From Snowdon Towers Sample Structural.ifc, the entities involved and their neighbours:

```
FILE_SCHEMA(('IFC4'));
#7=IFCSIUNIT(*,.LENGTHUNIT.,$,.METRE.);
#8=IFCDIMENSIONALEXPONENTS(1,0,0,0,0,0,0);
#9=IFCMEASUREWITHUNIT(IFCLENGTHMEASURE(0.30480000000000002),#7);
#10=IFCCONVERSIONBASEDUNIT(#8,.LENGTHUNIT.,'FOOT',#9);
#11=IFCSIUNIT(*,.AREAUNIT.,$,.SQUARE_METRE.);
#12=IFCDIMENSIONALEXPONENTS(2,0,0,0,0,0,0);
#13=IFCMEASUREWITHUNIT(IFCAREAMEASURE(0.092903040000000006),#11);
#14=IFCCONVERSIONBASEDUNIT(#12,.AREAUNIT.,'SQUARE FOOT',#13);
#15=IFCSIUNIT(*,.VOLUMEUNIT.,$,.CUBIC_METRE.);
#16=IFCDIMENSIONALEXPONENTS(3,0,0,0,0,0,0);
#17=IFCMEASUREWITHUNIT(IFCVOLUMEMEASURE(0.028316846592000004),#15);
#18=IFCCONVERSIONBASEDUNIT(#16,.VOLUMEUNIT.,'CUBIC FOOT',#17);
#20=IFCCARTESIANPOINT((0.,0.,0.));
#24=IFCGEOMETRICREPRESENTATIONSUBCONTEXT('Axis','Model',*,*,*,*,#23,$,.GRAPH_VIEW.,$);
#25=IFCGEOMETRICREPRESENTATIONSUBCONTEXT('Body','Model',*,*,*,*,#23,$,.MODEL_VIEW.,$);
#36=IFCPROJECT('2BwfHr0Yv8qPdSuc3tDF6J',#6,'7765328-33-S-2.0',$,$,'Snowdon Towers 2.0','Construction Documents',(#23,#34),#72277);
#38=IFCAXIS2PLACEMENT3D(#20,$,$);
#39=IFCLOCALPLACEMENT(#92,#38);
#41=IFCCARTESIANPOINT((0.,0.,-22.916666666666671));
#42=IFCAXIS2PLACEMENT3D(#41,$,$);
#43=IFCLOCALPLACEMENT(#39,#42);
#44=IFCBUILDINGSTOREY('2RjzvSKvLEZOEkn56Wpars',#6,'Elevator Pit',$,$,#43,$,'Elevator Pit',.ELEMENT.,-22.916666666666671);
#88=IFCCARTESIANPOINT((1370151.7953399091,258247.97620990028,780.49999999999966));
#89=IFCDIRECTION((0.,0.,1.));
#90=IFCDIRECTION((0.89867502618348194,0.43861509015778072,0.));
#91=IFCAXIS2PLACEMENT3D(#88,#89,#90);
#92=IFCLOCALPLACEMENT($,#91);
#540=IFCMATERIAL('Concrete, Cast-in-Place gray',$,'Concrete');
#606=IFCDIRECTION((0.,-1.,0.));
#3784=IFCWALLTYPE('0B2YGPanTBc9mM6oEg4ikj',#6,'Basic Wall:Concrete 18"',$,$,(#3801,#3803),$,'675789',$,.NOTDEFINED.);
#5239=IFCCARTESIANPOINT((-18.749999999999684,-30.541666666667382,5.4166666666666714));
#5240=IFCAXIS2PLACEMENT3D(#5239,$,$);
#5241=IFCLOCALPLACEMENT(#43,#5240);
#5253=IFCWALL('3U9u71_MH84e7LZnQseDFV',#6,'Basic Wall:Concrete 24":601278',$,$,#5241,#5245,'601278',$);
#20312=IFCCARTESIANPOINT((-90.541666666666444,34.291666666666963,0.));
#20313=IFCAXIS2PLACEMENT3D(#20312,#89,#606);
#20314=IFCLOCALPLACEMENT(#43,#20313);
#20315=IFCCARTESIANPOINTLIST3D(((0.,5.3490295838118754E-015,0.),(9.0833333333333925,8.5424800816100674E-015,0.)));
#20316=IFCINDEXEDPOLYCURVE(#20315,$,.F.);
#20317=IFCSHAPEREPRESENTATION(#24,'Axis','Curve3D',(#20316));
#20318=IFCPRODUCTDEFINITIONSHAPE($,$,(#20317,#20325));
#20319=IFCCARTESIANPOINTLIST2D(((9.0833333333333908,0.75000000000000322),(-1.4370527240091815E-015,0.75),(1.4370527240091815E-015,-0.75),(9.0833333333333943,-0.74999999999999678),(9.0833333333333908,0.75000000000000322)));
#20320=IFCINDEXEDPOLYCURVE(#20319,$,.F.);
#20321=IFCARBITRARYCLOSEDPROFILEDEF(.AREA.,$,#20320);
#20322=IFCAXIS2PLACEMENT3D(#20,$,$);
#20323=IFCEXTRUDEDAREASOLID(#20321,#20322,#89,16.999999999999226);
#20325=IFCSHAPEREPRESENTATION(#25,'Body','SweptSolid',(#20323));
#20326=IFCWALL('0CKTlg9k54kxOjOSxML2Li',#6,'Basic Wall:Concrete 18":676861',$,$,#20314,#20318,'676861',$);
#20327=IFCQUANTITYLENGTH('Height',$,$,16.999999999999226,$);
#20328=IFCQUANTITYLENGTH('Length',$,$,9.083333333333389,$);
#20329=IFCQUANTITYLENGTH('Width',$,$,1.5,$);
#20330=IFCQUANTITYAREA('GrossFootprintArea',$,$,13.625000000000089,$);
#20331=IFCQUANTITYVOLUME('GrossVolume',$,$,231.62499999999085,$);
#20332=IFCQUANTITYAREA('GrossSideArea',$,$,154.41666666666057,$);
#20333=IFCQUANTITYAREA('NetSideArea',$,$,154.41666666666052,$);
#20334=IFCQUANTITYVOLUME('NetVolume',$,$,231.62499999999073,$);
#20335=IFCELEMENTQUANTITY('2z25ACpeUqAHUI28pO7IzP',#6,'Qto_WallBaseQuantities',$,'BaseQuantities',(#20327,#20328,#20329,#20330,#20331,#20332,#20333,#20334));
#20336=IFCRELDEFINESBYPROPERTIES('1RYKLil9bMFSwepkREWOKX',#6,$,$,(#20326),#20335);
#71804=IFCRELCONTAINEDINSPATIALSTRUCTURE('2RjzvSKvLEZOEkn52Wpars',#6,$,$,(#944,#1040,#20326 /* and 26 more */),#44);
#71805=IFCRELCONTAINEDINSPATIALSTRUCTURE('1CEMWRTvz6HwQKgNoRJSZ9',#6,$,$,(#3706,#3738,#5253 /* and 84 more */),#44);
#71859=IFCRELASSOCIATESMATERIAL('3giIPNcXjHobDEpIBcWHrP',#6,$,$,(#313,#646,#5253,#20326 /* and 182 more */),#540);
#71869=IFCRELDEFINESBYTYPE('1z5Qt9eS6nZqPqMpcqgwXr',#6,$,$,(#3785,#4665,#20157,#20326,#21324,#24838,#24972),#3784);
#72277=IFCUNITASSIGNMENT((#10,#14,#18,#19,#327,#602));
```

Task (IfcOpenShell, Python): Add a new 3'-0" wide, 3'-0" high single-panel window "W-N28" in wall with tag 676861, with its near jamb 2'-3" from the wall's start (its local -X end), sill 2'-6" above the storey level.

```python
import numpy as np
import ifcopenshell
import ifcopenshell.api.feature
import ifcopenshell.api.geometry
import ifcopenshell.api.pset
import ifcopenshell.api.root
import ifcopenshell.api.spatial
import ifcopenshell.geom
import ifcopenshell.util.element
import ifcopenshell.util.placement
import ifcopenshell.util.representation
import ifcopenshell.util.shape
import ifcopenshell.util.unit

model = ifcopenshell.open("Snowdon Towers Sample Structural.ifc")
unit_scale = ifcopenshell.util.unit.calculate_unit_scale(model)
area_scale = ifcopenshell.util.unit.calculate_unit_scale(model, "AREAUNIT")
volume_scale = ifcopenshell.util.unit.calculate_unit_scale(model, "VOLUMEUNIT")
settings = ifcopenshell.geom.settings()


def volume(element):
    """Net volume in cubic metres, openings subtracted."""
    shape = ifcopenshell.geom.create_shape(settings, element)
    return ifcopenshell.util.shape.get_volume(shape.geometry)


wall = model.by_guid("0CKTlg9k54kxOjOSxML2Li")
storey = ifcopenshell.util.element.get_container(wall, ifc_class="IfcBuildingStorey")
context = ifcopenshell.util.representation.get_context(model, "Model", "Body", "MODEL_VIEW")
before = volume(wall)

width, height, from_end, sill = 0.9144, 0.9144, 0.6858, 0.762  # metres

# The wall runs along its own X axis, and the end named is its -X end.
wall_shape = ifcopenshell.geom.create_shape(settings, wall)
x, y, z = ifcopenshell.util.shape.get_vertices(wall_shape.geometry).T
start = x.min() + from_end
face, thickness = float(y.min()), float(y.max() - y.min())
wall_matrix = ifcopenshell.util.placement.get_local_placement(wall.ObjectPlacement)
level = ifcopenshell.util.placement.get_local_placement(storey.ObjectPlacement)[2, 3]


def in_wall(x, y):
    """Placement at x, y metres in the wall's axes, at sill height."""
    matrix = wall_matrix.copy()
    matrix[:, 3] = wall_matrix @ np.array([x / unit_scale, y / unit_scale, 0.0, 1.0])
    matrix[2, 3] = level + sill / unit_scale
    return matrix


# Opening: a box that overshoots both wall faces by 50 mm.
opening = ifcopenshell.api.root.create_entity(model, ifc_class="IfcOpeningElement", predefined_type="OPENING")
box = ifcopenshell.api.geometry.add_wall_representation(
    model, context=context, length=width, height=height, thickness=thickness + 0.1
)
ifcopenshell.api.geometry.assign_representation(model, product=opening, representation=box)
ifcopenshell.api.geometry.edit_object_placement(model, product=opening, matrix=in_wall(start, face - 0.05), is_si=False)
ifcopenshell.api.feature.add_feature(model, feature=opening, element=wall)

window = ifcopenshell.api.root.create_entity(model, ifc_class="IfcWindow", name="W-N28", predefined_type="WINDOW")
window.OverallWidth, window.OverallHeight = width / unit_scale, height / unit_scale
window.PartitioningType = "SINGLE_PANEL"
body = ifcopenshell.api.geometry.add_window_representation(
    model,
    context=context,
    overall_width=window.OverallWidth,
    overall_height=window.OverallHeight,
    partition_type="SINGLE_PANEL",
)
ifcopenshell.api.geometry.assign_representation(model, product=window, representation=body)
ifcopenshell.api.spatial.assign_container(model, products=[window], relating_structure=storey)
ifcopenshell.api.feature.add_filling(model, opening=opening, element=window)

# Centre the window in the wall's thickness.
ifcopenshell.api.geometry.edit_object_placement(model, product=window, matrix=in_wall(start, face), is_si=False)
window_shape = ifcopenshell.geom.create_shape(settings, window)
depth = ifcopenshell.util.shape.get_vertices(window_shape.geometry)[:, 1]
offset = face + thickness / 2 - (depth.min() + depth.max()) / 2
ifcopenshell.api.geometry.edit_object_placement(model, product=window, matrix=in_wall(start, offset), is_si=False)

after = volume(wall)

# Update the wall's stored quantities.
qto = model.by_id(ifcopenshell.util.element.get_pset(wall, "Qto_WallBaseQuantities", should_inherit=False)["id"])
ifcopenshell.api.pset.edit_qto(model, qto=qto, properties={
    "NetSideArea": after / thickness / area_scale,
    "NetVolume": after / volume_scale,
})

print(f"wall volume {before:.3f} -> {after:.3f} m3")

model.write("Snowdon Towers Sample Structural-out.ifc")
```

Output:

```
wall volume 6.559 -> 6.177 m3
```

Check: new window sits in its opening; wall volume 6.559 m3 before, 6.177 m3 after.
